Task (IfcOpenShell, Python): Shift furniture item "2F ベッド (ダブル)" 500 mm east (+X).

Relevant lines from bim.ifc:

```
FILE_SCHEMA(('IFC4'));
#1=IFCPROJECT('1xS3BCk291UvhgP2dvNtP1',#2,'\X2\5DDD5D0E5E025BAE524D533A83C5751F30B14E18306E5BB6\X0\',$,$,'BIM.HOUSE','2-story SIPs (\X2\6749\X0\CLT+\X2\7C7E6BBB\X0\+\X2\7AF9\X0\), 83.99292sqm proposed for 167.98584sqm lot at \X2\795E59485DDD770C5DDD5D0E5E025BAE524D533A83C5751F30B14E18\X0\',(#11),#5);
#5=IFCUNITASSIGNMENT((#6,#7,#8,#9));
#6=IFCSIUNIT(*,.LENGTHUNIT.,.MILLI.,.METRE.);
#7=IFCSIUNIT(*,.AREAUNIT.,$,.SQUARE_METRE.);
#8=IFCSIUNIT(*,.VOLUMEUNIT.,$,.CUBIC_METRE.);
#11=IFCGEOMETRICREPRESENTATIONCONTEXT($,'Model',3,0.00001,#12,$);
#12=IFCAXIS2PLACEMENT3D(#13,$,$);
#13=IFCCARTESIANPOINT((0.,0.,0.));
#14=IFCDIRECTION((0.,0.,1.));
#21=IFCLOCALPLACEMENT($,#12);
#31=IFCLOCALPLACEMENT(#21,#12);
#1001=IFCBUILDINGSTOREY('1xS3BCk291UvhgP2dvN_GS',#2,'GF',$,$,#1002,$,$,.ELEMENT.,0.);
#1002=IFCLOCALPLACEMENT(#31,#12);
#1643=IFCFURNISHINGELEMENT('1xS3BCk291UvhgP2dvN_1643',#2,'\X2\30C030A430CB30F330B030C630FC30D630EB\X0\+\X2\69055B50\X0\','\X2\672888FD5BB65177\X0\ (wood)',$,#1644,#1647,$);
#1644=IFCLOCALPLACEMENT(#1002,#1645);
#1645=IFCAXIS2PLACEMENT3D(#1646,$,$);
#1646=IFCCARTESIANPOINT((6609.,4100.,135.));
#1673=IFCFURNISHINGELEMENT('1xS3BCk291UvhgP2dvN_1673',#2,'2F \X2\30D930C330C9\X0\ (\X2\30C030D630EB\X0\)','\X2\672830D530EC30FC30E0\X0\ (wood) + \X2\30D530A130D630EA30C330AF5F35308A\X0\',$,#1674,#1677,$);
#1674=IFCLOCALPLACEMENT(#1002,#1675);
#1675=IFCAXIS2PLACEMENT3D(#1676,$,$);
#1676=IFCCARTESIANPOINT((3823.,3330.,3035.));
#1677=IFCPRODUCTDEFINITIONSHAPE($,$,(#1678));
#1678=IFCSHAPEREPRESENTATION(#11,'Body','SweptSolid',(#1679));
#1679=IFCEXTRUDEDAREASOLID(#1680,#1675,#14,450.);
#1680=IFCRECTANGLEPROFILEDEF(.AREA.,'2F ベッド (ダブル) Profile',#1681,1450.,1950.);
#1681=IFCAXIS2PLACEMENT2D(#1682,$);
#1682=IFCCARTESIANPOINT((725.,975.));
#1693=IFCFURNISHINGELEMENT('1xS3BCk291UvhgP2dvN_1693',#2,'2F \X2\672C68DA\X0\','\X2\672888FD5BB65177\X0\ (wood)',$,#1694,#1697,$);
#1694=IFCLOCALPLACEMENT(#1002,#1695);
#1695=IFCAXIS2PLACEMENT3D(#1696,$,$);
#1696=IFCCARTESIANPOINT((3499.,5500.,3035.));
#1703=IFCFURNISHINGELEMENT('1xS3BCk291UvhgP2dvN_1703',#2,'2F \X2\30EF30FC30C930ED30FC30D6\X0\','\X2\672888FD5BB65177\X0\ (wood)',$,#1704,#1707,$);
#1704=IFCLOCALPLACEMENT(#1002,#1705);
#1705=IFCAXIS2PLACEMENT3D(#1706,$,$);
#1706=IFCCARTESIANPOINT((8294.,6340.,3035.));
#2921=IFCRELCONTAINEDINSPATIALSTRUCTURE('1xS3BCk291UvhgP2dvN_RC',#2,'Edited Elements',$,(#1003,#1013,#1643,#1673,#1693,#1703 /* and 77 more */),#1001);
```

```python
import ifcopenshell
import ifcopenshell.api.geometry
import ifcopenshell.util.placement
import ifcopenshell.util.unit

model = ifcopenshell.open("bim.ifc")
unit_scale = ifcopenshell.util.unit.calculate_unit_scale(model)

item = model.by_guid("1xS3BCk291UvhgP2dvN_1673")
matrix = ifcopenshell.util.placement.get_local_placement(item.ObjectPlacement)
matrix[0, 3] += 0.5 / unit_scale
ifcopenshell.api.geometry.edit_object_placement(model, product=item, matrix=matrix, is_si=False)

print(ifcopenshell.util.placement.get_local_placement(item.ObjectPlacement).round(3) + 0.0)

model.write("bim_edited.ifc")
```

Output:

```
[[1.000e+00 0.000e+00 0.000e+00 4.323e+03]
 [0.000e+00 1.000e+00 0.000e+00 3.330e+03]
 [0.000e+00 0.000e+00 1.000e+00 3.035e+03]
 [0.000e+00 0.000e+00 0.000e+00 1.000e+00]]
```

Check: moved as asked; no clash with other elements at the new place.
